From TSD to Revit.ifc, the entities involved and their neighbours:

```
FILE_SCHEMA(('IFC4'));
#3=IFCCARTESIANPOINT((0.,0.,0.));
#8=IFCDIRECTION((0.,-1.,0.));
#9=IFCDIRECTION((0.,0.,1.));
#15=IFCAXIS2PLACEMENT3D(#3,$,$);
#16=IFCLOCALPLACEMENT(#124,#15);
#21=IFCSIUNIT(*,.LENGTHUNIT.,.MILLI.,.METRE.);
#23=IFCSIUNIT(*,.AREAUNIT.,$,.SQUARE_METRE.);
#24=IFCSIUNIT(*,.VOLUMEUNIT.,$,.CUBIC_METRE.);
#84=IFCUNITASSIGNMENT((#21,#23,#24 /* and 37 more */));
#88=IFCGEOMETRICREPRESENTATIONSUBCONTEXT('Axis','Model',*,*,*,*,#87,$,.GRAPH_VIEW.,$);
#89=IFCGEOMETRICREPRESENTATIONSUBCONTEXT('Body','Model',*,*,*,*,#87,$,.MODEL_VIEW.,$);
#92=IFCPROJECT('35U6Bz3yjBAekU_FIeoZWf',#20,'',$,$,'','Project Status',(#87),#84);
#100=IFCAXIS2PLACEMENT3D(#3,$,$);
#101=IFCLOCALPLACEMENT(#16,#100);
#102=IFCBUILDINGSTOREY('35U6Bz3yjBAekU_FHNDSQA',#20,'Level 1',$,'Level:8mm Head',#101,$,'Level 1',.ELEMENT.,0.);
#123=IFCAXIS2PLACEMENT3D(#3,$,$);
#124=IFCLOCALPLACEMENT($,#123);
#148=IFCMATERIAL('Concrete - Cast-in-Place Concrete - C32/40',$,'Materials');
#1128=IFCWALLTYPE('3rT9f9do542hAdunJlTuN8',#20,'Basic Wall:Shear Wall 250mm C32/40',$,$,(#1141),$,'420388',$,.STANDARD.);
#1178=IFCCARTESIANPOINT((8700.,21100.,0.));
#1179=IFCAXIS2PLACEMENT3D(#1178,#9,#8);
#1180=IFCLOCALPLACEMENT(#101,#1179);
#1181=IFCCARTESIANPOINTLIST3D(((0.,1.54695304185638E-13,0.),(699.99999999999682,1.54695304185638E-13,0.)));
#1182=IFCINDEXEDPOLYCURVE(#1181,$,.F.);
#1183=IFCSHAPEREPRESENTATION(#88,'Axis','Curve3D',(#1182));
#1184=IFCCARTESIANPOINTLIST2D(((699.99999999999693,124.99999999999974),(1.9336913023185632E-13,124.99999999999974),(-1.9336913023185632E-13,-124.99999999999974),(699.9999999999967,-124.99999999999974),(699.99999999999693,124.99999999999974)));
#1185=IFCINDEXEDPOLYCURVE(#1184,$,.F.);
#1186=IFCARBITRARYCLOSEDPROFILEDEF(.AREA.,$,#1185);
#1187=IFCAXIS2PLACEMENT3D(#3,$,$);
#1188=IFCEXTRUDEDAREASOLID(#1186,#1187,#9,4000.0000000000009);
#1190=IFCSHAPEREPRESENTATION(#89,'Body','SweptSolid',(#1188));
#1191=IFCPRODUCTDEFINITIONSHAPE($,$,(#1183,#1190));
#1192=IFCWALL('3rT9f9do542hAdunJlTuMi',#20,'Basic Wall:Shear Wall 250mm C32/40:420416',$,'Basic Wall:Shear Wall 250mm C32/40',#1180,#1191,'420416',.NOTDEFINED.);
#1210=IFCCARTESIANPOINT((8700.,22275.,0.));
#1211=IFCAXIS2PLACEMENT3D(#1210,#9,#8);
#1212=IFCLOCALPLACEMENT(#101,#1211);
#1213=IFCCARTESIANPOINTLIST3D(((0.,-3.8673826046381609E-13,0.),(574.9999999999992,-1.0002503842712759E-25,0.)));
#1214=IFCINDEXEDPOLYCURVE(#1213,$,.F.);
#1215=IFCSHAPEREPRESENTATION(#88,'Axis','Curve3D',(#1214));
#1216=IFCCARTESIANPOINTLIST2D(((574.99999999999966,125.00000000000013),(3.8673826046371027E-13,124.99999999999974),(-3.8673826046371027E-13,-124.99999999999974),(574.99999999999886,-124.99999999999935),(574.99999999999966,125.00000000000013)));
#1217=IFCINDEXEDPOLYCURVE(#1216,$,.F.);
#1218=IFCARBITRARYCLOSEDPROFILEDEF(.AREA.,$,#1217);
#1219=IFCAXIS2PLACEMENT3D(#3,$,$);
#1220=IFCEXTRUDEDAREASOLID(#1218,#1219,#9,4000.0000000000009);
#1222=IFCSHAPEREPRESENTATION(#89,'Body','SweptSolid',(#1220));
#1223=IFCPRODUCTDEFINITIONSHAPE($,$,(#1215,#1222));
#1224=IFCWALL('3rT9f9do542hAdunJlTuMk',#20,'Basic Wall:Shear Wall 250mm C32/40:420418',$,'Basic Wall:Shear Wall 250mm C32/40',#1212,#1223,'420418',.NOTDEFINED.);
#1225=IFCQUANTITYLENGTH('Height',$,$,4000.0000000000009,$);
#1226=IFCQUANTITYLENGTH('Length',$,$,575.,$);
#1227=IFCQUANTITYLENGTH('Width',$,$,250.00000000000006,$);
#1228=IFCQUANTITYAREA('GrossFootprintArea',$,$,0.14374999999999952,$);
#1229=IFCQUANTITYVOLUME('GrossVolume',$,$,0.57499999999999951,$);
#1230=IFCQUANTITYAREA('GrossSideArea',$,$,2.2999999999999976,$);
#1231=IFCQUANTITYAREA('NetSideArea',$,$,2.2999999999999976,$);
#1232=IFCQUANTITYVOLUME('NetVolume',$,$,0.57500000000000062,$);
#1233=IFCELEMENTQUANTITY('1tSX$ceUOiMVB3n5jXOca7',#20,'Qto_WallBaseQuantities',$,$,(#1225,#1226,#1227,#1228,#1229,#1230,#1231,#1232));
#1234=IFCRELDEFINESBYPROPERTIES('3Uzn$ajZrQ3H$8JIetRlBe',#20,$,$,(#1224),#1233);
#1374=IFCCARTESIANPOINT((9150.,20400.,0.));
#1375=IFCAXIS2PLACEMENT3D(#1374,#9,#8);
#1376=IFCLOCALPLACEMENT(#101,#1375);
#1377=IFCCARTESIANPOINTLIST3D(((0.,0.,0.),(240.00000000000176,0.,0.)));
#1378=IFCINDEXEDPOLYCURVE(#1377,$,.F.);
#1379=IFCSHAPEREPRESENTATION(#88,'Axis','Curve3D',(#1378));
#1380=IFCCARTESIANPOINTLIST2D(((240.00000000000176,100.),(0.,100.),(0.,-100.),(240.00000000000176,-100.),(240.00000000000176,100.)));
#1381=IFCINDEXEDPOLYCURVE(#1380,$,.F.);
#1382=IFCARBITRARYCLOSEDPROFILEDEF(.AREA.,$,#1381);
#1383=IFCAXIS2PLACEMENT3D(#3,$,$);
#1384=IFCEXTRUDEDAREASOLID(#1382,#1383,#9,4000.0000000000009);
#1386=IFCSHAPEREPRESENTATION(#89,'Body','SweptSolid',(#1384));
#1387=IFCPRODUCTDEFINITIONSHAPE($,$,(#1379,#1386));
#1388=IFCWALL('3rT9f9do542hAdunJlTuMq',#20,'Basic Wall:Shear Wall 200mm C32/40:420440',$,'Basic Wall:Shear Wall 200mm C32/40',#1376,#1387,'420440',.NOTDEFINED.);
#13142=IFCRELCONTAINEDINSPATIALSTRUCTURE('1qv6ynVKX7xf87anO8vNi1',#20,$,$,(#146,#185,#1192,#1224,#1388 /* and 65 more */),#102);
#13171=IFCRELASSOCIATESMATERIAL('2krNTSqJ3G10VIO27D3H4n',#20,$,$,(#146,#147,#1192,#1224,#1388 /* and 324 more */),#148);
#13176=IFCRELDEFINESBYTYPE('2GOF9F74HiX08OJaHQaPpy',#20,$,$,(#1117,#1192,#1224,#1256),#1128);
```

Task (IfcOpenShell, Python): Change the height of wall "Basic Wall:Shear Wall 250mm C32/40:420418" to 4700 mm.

```python
import ifcopenshell
import ifcopenshell.api.pset
import ifcopenshell.geom
import ifcopenshell.util.element
import ifcopenshell.util.representation
import ifcopenshell.util.shape
import ifcopenshell.util.unit

model = ifcopenshell.open("TSD to Revit.ifc")
unit_scale = ifcopenshell.util.unit.calculate_unit_scale(model)
area_scale = ifcopenshell.util.unit.calculate_unit_scale(model, "AREAUNIT")
volume_scale = ifcopenshell.util.unit.calculate_unit_scale(model, "VOLUMEUNIT")
settings = ifcopenshell.geom.settings()


def volume(element):
    """Net volume in cubic metres, openings subtracted."""
    shape = ifcopenshell.geom.create_shape(settings, element)
    return ifcopenshell.util.shape.get_volume(shape.geometry)


wall = model.by_guid("3rT9f9do542hAdunJlTuMk")
before = volume(wall)

body = ifcopenshell.util.representation.get_representation(wall, "Model", "Body")
solid = body.Items[0]
old_height = solid.Depth
solid.Depth = 4.7 / unit_scale
after = volume(wall)
thickness = 0.25  # wall thickness in metres

# Update the stored height, areas and volumes.
qto = model.by_id(ifcopenshell.util.element.get_pset(wall, "Qto_WallBaseQuantities", should_inherit=False)["id"])
ifcopenshell.api.pset.edit_qto(model, qto=qto, properties={
    "Height": solid.Depth,
    "GrossVolume": ifcopenshell.util.element.get_pset(wall, "Qto_WallBaseQuantities", "GrossVolume") * solid.Depth / old_height,
    "GrossSideArea": ifcopenshell.util.element.get_pset(wall, "Qto_WallBaseQuantities", "GrossSideArea") * solid.Depth / old_height,
    "NetSideArea": after / thickness / area_scale,
    "NetVolume": after / volume_scale,
})

print(f"height {old_height:g} -> {solid.Depth:g}, volume {before:.3f} -> {after:.3f} m3")

model.write("TSD to Revit-out.ifc")
```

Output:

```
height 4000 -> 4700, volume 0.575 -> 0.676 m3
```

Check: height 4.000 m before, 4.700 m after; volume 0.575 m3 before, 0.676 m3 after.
